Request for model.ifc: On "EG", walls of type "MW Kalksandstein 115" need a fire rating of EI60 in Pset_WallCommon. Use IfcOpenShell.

First a look at what the model holds.

```python
import ifcopenshell
import ifcopenshell.util.element

model = ifcopenshell.open("model.ifc")
print(model.schema)
storey = next(s for s in model.by_type("IfcBuildingStorey") if s.Name == "EG")
walls = [e for e in ifcopenshell.util.element.get_decomposition(storey) if e.is_a("IfcWall")]
seen = {}
for e in walls:
    element_type = ifcopenshell.util.element.get_type(e)
    key = (element_type.Name if element_type != e and element_type else None, ifcopenshell.util.element.get_pset(e, "Pset_WallCommon", "FireRating"))
    seen[key] = seen.get(key, 0) + 1
for (name, value), count in sorted(seen.items(), key=str):
    print(count, "x", name, "|", value)
```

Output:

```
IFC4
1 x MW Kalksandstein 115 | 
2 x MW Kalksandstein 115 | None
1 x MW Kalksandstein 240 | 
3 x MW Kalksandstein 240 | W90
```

```python
import ifcopenshell
import ifcopenshell.api.pset
import ifcopenshell.util.element

model = ifcopenshell.open("model.ifc")

storey = next(s for s in model.by_type("IfcBuildingStorey") if s.Name == "EG")
walls = [e for e in ifcopenshell.util.element.get_decomposition(storey) if e.is_a("IfcWall")]

count = 0
for e in walls:
    element_type = ifcopenshell.util.element.get_type(e)
    if element_type in (None, e) or element_type.Name != "MW Kalksandstein 115":
        continue
    # add_pset returns the element's existing set when there is one.
    pset = ifcopenshell.api.pset.add_pset(model, product=e, name="Pset_WallCommon")
    ifcopenshell.api.pset.edit_pset(model, pset=pset, properties={"FireRating": "EI60"})
    count += 1

print(count, "walls updated")

model.write("model-out.ifc")
```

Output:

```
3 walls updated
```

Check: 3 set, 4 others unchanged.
